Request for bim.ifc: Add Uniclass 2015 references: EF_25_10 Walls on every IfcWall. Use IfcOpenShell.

First a look at what the model holds.

```python
import ifcopenshell

model = ifcopenshell.open("bim.ifc")
print(model.schema)
print("classifications:", [c.Name for c in model.by_type("IfcClassification")])
for ifc_class in ("IfcDoor", "IfcRoof", "IfcStair", "IfcWall", "IfcWindow"):
    print(ifc_class, len(model.by_type(ifc_class)))
```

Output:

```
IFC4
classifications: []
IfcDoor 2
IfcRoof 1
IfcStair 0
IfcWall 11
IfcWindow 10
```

```python
import ifcopenshell
import ifcopenshell.api.classification

model = ifcopenshell.open("bim.ifc")

system = ifcopenshell.api.classification.add_classification(model, classification="Uniclass 2015")

codes = {
    "IfcWall": ("EF_25_10", "Walls"),
}
for ifc_class, (code, name) in codes.items():
    products = model.by_type(ifc_class)
    ifcopenshell.api.classification.add_reference(
        model, products=products, classification=system, identification=code, name=name
    )
    print(code, len(products))

model.write("bim_rev.ifc")
```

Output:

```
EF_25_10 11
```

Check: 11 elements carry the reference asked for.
